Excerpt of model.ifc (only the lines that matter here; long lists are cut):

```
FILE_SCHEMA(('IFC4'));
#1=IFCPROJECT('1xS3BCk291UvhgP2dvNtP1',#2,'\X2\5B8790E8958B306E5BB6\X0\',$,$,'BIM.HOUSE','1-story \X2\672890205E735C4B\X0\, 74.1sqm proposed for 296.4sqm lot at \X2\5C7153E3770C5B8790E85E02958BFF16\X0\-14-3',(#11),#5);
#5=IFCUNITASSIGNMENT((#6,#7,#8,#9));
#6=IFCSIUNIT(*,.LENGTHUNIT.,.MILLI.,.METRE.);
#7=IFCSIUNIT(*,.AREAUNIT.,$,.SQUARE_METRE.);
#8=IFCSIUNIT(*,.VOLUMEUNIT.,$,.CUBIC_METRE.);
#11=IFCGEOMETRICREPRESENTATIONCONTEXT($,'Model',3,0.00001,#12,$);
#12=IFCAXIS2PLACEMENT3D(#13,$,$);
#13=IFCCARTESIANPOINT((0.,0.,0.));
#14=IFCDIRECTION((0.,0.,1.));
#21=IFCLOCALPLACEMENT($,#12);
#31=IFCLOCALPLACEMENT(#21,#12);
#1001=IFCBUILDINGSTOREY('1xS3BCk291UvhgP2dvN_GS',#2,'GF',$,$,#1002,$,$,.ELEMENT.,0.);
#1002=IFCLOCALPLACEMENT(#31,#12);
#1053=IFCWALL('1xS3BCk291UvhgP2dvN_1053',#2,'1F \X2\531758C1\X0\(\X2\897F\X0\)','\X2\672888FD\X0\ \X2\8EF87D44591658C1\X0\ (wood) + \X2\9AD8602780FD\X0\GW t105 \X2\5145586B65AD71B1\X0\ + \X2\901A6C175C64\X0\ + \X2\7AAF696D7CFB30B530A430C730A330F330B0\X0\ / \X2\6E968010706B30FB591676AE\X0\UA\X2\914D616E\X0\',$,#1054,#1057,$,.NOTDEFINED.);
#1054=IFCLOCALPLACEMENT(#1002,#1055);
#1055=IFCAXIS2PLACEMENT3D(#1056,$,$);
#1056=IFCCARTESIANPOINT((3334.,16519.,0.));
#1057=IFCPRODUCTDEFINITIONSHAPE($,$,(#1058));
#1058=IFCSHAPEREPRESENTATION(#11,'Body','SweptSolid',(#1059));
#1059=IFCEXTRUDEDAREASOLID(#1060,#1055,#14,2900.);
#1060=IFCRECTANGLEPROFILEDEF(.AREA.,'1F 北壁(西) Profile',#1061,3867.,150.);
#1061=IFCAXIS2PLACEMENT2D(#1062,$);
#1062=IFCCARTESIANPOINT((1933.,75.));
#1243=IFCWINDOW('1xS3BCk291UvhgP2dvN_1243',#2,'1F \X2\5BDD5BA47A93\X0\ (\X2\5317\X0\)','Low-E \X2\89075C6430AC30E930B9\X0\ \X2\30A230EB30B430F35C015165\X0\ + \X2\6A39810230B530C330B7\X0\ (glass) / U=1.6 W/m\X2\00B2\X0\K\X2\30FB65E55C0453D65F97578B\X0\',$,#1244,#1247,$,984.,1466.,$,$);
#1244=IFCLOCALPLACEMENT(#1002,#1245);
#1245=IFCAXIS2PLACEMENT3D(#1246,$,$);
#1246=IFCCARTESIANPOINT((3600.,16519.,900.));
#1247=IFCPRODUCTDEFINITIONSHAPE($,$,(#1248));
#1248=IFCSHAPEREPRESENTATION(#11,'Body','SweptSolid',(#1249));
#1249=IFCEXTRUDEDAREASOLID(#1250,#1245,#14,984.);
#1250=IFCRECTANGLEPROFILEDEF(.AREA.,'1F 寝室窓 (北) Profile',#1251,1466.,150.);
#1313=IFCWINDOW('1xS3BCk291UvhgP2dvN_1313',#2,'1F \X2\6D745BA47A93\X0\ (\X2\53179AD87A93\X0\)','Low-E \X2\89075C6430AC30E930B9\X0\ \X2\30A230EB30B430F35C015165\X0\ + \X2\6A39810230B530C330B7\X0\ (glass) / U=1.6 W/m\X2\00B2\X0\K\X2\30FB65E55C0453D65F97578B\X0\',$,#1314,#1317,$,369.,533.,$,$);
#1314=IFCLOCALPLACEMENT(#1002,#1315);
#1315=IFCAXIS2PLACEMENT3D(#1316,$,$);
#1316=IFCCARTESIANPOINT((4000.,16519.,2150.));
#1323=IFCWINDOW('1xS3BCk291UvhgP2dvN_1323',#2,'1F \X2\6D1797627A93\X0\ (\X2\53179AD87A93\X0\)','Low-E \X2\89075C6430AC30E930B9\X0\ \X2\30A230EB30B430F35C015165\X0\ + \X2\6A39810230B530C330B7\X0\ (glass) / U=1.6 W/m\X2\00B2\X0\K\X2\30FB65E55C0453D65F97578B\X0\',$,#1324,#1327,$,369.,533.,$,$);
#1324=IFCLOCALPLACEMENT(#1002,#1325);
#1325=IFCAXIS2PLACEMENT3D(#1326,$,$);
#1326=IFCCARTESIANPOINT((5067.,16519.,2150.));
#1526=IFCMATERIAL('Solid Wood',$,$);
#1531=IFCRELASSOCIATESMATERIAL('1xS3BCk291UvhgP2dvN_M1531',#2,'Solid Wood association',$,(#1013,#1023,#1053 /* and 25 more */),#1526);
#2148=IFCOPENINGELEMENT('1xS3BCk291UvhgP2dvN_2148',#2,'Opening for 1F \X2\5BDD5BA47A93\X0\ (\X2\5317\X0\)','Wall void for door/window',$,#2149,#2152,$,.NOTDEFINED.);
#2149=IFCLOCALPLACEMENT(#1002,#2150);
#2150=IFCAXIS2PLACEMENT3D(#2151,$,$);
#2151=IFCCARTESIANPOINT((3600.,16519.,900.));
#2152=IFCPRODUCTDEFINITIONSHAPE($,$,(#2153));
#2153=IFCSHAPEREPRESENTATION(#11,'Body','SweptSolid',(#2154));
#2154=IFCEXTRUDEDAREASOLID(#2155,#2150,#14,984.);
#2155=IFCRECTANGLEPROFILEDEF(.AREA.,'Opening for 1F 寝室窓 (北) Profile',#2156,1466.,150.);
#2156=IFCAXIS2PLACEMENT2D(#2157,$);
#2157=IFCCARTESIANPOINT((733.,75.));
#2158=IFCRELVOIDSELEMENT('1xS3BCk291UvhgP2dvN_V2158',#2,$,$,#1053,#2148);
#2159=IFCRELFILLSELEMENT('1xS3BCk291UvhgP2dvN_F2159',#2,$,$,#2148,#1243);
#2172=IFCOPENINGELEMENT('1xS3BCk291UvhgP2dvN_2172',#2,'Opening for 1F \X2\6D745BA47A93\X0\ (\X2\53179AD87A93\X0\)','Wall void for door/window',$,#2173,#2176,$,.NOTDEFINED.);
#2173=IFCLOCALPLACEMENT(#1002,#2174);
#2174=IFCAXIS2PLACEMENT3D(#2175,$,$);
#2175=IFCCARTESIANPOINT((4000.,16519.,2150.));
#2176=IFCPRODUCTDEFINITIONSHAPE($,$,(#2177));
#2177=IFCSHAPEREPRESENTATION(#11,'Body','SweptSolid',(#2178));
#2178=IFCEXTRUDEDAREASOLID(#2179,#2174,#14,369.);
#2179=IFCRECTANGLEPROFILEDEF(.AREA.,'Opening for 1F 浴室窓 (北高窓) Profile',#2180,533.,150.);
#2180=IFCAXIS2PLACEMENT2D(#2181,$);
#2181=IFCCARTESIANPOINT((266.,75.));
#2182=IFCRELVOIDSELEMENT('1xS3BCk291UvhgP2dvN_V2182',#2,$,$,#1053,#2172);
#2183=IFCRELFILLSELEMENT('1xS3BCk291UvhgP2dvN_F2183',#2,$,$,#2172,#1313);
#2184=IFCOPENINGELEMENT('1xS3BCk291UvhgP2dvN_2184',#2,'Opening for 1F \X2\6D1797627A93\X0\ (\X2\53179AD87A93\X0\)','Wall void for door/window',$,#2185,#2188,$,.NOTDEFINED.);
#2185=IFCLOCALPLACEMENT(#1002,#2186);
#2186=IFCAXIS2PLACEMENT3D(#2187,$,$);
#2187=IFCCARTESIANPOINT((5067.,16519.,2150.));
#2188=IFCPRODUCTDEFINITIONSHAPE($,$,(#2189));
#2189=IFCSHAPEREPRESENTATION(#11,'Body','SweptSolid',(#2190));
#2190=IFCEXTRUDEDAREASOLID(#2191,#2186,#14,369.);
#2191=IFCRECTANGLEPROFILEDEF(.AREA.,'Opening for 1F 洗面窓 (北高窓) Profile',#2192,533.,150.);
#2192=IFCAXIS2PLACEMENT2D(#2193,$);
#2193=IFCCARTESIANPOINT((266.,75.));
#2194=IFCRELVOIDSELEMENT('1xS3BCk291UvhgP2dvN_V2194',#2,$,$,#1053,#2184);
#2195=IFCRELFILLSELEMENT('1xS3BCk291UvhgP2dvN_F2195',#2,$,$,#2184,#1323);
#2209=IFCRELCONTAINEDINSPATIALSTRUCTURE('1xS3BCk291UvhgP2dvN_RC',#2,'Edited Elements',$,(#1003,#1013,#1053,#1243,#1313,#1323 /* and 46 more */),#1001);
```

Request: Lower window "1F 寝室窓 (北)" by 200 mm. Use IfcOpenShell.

```python
import numpy as np
import ifcopenshell
import ifcopenshell.api.geometry
import ifcopenshell.util.placement
import ifcopenshell.util.unit

model = ifcopenshell.open("model.ifc")
unit_scale = ifcopenshell.util.unit.calculate_unit_scale(model)

window = model.by_guid("1xS3BCk291UvhgP2dvN_1243")
opening = window.FillsVoids[0].RelatingOpeningElement
dz = -0.2 / unit_scale

shift = np.array([0.0, 0.0, dz])
# The window is not placed relative to its opening, so move both.
for product in (opening, window):
    matrix = ifcopenshell.util.placement.get_local_placement(product.ObjectPlacement)
    matrix[:3, 3] += shift
    ifcopenshell.api.geometry.edit_object_placement(model, product=product, matrix=matrix, is_si=False)

print(f"moved by {dz * unit_scale:+.3f} m")

model.write("model_v2.ifc")
```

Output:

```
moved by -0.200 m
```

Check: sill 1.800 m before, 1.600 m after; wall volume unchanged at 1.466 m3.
